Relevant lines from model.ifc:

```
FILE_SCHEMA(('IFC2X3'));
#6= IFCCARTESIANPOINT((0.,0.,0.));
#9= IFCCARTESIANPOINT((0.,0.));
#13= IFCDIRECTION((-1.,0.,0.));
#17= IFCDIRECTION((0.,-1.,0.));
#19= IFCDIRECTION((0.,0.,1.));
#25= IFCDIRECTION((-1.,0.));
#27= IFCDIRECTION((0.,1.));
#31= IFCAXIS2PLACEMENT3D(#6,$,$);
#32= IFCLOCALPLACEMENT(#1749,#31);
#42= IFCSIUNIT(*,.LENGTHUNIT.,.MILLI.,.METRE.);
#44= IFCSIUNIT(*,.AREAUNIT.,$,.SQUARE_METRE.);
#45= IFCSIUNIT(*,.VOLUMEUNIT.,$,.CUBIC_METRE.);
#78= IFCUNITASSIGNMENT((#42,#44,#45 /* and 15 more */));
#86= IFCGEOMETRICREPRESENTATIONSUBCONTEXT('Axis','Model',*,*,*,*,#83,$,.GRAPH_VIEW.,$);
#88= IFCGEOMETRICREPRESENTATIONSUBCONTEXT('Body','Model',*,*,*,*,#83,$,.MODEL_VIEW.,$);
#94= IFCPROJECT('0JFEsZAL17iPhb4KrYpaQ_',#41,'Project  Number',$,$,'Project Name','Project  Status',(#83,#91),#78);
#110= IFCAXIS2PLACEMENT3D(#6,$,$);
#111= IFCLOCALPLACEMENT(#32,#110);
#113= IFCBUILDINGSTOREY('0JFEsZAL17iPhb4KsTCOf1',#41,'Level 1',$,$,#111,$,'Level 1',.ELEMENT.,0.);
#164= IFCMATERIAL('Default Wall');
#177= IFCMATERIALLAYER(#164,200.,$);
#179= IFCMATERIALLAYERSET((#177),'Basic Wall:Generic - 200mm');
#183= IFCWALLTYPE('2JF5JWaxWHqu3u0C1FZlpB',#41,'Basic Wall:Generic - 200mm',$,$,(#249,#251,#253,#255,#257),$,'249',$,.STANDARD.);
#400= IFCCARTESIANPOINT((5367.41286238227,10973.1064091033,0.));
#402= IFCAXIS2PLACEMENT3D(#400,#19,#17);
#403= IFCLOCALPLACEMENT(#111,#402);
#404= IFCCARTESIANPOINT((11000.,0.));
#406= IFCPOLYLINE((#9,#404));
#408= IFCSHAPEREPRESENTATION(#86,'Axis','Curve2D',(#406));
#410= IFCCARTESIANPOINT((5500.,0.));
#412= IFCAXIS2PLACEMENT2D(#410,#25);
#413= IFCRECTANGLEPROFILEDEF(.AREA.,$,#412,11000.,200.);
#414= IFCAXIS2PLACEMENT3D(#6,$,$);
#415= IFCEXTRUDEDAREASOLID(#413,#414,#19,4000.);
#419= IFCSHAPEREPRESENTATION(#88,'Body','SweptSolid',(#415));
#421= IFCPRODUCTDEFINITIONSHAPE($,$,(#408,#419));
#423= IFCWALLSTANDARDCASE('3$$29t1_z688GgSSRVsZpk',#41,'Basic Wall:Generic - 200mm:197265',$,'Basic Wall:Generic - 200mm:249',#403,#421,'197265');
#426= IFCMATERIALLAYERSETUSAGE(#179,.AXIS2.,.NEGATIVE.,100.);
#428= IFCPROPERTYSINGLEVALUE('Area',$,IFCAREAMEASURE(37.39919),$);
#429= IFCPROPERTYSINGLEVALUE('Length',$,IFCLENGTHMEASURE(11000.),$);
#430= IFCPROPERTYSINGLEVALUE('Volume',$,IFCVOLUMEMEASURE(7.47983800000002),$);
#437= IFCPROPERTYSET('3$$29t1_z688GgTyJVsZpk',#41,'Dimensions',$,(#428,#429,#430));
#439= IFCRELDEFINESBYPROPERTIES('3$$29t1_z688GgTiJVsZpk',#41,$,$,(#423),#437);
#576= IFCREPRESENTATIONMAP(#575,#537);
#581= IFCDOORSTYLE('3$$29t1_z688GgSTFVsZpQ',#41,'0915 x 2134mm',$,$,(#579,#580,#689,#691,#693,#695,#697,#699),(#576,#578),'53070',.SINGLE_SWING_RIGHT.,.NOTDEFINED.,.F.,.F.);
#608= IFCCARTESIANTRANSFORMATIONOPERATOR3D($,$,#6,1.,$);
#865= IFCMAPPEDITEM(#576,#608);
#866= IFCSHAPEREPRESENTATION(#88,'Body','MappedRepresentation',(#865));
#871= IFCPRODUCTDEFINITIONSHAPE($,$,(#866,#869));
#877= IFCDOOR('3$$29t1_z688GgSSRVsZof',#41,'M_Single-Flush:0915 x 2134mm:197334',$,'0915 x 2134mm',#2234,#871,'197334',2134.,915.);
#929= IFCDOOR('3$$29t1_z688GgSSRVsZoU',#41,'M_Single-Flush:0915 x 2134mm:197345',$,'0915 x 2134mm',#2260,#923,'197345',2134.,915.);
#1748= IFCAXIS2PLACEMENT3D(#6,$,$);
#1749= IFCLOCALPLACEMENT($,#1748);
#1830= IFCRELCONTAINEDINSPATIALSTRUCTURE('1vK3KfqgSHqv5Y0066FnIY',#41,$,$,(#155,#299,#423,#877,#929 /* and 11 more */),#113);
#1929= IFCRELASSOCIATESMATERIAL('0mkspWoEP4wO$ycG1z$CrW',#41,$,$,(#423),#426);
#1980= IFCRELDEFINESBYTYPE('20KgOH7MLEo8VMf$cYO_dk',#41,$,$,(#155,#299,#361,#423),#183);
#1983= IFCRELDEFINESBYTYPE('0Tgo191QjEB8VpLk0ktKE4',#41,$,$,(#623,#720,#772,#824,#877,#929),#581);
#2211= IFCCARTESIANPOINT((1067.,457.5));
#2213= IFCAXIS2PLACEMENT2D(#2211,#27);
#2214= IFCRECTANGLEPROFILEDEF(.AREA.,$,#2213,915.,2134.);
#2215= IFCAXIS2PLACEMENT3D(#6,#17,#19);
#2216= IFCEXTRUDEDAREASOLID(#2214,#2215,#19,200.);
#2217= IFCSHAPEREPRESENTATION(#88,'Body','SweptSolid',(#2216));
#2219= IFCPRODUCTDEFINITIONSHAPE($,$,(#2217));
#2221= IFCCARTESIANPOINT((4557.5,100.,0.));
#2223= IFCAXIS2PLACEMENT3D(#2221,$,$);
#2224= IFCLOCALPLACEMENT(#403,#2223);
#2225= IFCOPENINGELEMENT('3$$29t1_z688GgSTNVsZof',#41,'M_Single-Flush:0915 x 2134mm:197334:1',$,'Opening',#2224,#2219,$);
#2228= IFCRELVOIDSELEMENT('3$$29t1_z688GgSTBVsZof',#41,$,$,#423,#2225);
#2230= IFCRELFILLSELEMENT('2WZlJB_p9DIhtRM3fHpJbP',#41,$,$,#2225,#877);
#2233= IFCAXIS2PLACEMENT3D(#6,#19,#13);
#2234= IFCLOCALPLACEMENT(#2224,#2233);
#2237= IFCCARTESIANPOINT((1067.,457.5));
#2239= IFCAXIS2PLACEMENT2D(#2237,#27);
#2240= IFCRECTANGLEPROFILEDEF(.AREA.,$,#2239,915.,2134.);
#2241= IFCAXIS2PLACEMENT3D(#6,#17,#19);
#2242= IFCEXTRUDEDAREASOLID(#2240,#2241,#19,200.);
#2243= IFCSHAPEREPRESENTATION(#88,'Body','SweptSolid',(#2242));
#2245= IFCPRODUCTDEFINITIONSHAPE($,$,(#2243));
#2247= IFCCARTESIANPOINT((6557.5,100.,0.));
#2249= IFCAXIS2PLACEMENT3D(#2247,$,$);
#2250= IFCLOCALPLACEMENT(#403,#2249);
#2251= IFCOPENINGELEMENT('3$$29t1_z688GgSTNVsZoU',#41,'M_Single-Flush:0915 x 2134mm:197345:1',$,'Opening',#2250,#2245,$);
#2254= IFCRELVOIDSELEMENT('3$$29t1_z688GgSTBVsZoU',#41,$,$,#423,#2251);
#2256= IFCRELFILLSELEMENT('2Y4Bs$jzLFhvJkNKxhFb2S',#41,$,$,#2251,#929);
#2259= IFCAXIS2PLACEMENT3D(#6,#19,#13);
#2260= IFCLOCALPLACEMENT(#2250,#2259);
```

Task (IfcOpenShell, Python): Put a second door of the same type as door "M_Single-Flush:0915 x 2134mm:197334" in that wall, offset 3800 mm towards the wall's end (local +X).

```python
import ifcopenshell
import ifcopenshell.api.feature
import ifcopenshell.api.geometry
import ifcopenshell.api.pset
import ifcopenshell.api.root
import ifcopenshell.geom
import ifcopenshell.util.element
import ifcopenshell.util.placement
import ifcopenshell.util.shape
import ifcopenshell.util.unit

model = ifcopenshell.open("model.ifc")
unit_scale = ifcopenshell.util.unit.calculate_unit_scale(model)
area_scale = ifcopenshell.util.unit.calculate_unit_scale(model, "AREAUNIT")
volume_scale = ifcopenshell.util.unit.calculate_unit_scale(model, "VOLUMEUNIT")
settings = ifcopenshell.geom.settings()


def volume(element):
    """Net volume in cubic metres, openings subtracted."""
    shape = ifcopenshell.geom.create_shape(settings, element)
    return ifcopenshell.util.shape.get_volume(shape.geometry)


def reuse_history(source, copy):
    """copy_class also copies each property set's owner history, people and application; keep the originals."""
    for rel in copy.IsDefinedBy:
        if rel.is_a("IfcRelDefinesByProperties") and (history := rel.RelatingPropertyDefinition.OwnerHistory):
            rel.RelatingPropertyDefinition.OwnerHistory = source.OwnerHistory
            ifcopenshell.util.element.remove_deep2(model, history)


door = model.by_guid("3$$29t1_z688GgSSRVsZof")
opening = door.FillsVoids[0].RelatingOpeningElement
wall = opening.VoidsElements[0].RelatingBuildingElement
before = volume(wall)
shift = ifcopenshell.util.placement.get_local_placement(wall.ObjectPlacement)[:3, 0] * 3.8 / unit_scale

# copy_class copies the void relationship, type, container and properties, but no geometry.
new_opening = ifcopenshell.api.root.copy_class(model, product=opening)
new_opening.Representation = ifcopenshell.util.element.copy_deep(
    model, opening.Representation, exclude=["IfcGeometricRepresentationContext", "IfcRepresentationMap"]
)
new_opening.Name = "M_Single-Flush:0915 x 2134mm"
new_door = ifcopenshell.api.root.copy_class(model, product=door)
new_door.Representation = ifcopenshell.util.element.copy_deep(
    model, door.Representation, exclude=["IfcGeometricRepresentationContext", "IfcRepresentationMap"]
)
new_door.Name = "M_Single-Flush:0915 x 2134mm"
new_door.Tag = None
reuse_history(door, new_door)
fills = ifcopenshell.api.feature.add_filling(model, opening=new_opening, element=new_door)
fills.OwnerHistory = new_door.OwnerHistory  # required in IFC2X3

for old, new in ((opening, new_opening), (door, new_door)):
    matrix = ifcopenshell.util.placement.get_local_placement(old.ObjectPlacement)
    matrix[:3, 3] += shift
    ifcopenshell.api.geometry.edit_object_placement(model, product=new, matrix=matrix, is_si=False)

after = volume(wall)
thickness = 0.2  # wall thickness in metres

# Update the wall's stored quantities.
pset = model.by_id(ifcopenshell.util.element.get_pset(wall, "Dimensions", should_inherit=False)["id"])
ifcopenshell.api.pset.edit_pset(model, pset=pset, properties={
    "Area": model.create_entity("IfcAreaMeasure", after / thickness / area_scale),
    "Volume": model.create_entity("IfcVolumeMeasure", after / volume_scale),
})

print(f"wall volume {before:.3f} -> {after:.3f} m3")

model.write("model-out.ifc")
```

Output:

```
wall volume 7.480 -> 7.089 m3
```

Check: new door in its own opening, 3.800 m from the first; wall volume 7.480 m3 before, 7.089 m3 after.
